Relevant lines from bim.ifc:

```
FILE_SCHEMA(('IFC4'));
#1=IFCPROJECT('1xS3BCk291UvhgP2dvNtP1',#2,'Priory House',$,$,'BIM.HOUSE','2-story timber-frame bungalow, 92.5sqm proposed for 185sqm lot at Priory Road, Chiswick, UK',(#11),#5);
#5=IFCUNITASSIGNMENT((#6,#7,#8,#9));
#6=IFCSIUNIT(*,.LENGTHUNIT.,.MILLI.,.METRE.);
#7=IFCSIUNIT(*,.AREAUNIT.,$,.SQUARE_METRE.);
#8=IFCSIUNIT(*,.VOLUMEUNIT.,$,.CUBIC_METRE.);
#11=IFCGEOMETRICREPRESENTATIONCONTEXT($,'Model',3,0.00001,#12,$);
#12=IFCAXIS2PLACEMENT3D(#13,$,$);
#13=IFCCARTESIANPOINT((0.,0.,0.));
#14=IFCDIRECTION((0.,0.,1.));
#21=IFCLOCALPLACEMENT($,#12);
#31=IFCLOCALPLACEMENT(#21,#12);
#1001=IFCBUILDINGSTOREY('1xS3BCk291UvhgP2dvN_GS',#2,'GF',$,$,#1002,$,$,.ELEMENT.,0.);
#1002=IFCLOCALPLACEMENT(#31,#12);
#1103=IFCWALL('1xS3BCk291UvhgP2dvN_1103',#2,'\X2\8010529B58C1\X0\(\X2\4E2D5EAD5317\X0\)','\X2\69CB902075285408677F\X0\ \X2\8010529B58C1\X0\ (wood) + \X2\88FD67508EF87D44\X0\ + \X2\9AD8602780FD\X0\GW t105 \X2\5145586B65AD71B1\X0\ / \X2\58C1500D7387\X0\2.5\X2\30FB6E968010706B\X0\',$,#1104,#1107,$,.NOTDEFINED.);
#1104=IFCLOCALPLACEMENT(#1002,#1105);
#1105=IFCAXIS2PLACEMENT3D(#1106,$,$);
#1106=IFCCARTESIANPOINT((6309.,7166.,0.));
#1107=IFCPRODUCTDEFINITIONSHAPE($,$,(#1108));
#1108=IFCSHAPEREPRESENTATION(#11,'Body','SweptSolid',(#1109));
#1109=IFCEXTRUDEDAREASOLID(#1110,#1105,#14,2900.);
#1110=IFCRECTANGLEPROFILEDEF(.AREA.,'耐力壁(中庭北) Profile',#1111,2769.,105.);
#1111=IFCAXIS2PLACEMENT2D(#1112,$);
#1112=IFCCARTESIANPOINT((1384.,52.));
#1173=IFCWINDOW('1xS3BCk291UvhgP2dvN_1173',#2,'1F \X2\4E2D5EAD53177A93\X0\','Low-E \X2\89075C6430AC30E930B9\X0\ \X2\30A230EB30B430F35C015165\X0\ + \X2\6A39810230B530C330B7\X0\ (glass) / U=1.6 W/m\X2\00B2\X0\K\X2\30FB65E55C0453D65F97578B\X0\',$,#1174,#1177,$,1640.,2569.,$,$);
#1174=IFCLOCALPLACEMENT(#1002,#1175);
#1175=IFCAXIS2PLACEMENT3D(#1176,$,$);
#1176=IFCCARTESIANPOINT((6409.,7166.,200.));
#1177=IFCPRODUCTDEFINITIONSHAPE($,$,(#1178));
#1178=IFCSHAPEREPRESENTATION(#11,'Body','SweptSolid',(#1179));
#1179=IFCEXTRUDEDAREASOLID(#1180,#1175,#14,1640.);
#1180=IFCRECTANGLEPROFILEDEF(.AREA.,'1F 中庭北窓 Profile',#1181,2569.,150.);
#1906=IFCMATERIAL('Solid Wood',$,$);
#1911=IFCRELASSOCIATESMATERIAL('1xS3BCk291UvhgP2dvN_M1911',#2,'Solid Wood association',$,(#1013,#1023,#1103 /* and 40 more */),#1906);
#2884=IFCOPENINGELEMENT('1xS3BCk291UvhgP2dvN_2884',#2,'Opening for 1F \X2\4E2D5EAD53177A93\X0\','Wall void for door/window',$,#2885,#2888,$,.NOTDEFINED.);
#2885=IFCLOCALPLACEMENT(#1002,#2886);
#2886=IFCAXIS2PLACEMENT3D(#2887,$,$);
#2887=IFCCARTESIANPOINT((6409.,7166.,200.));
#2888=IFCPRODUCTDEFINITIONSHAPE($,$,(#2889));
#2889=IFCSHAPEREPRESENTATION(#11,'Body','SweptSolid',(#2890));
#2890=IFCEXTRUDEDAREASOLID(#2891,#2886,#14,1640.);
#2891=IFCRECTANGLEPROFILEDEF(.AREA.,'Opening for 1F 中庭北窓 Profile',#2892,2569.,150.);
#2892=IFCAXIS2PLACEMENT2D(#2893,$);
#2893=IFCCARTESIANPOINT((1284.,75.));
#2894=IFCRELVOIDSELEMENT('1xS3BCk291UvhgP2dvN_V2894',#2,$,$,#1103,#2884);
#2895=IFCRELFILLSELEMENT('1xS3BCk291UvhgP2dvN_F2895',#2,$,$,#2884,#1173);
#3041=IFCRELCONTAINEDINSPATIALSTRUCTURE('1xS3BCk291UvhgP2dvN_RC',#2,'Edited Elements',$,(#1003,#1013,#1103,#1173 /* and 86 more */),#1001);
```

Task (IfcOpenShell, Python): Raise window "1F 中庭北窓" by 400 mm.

```python
import numpy as np
import ifcopenshell
import ifcopenshell.api.geometry
import ifcopenshell.util.placement
import ifcopenshell.util.unit

model = ifcopenshell.open("bim.ifc")
unit_scale = ifcopenshell.util.unit.calculate_unit_scale(model)

window = model.by_id(1173)
opening = window.FillsVoids[0].RelatingOpeningElement
dz = 400.0

shift = np.array([0.0, 0.0, dz])
# The window is not placed relative to its opening, so move both.
for product in (opening, window):
    matrix = ifcopenshell.util.placement.get_local_placement(product.ObjectPlacement)
    matrix[:3, 3] += shift
    ifcopenshell.api.geometry.edit_object_placement(model, product=product, matrix=matrix, is_si=False)

print(f"moved by {dz * unit_scale:+.3f} m")

model.write("bim_v2.ifc")
```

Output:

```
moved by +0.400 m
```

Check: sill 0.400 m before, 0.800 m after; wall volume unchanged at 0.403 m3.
